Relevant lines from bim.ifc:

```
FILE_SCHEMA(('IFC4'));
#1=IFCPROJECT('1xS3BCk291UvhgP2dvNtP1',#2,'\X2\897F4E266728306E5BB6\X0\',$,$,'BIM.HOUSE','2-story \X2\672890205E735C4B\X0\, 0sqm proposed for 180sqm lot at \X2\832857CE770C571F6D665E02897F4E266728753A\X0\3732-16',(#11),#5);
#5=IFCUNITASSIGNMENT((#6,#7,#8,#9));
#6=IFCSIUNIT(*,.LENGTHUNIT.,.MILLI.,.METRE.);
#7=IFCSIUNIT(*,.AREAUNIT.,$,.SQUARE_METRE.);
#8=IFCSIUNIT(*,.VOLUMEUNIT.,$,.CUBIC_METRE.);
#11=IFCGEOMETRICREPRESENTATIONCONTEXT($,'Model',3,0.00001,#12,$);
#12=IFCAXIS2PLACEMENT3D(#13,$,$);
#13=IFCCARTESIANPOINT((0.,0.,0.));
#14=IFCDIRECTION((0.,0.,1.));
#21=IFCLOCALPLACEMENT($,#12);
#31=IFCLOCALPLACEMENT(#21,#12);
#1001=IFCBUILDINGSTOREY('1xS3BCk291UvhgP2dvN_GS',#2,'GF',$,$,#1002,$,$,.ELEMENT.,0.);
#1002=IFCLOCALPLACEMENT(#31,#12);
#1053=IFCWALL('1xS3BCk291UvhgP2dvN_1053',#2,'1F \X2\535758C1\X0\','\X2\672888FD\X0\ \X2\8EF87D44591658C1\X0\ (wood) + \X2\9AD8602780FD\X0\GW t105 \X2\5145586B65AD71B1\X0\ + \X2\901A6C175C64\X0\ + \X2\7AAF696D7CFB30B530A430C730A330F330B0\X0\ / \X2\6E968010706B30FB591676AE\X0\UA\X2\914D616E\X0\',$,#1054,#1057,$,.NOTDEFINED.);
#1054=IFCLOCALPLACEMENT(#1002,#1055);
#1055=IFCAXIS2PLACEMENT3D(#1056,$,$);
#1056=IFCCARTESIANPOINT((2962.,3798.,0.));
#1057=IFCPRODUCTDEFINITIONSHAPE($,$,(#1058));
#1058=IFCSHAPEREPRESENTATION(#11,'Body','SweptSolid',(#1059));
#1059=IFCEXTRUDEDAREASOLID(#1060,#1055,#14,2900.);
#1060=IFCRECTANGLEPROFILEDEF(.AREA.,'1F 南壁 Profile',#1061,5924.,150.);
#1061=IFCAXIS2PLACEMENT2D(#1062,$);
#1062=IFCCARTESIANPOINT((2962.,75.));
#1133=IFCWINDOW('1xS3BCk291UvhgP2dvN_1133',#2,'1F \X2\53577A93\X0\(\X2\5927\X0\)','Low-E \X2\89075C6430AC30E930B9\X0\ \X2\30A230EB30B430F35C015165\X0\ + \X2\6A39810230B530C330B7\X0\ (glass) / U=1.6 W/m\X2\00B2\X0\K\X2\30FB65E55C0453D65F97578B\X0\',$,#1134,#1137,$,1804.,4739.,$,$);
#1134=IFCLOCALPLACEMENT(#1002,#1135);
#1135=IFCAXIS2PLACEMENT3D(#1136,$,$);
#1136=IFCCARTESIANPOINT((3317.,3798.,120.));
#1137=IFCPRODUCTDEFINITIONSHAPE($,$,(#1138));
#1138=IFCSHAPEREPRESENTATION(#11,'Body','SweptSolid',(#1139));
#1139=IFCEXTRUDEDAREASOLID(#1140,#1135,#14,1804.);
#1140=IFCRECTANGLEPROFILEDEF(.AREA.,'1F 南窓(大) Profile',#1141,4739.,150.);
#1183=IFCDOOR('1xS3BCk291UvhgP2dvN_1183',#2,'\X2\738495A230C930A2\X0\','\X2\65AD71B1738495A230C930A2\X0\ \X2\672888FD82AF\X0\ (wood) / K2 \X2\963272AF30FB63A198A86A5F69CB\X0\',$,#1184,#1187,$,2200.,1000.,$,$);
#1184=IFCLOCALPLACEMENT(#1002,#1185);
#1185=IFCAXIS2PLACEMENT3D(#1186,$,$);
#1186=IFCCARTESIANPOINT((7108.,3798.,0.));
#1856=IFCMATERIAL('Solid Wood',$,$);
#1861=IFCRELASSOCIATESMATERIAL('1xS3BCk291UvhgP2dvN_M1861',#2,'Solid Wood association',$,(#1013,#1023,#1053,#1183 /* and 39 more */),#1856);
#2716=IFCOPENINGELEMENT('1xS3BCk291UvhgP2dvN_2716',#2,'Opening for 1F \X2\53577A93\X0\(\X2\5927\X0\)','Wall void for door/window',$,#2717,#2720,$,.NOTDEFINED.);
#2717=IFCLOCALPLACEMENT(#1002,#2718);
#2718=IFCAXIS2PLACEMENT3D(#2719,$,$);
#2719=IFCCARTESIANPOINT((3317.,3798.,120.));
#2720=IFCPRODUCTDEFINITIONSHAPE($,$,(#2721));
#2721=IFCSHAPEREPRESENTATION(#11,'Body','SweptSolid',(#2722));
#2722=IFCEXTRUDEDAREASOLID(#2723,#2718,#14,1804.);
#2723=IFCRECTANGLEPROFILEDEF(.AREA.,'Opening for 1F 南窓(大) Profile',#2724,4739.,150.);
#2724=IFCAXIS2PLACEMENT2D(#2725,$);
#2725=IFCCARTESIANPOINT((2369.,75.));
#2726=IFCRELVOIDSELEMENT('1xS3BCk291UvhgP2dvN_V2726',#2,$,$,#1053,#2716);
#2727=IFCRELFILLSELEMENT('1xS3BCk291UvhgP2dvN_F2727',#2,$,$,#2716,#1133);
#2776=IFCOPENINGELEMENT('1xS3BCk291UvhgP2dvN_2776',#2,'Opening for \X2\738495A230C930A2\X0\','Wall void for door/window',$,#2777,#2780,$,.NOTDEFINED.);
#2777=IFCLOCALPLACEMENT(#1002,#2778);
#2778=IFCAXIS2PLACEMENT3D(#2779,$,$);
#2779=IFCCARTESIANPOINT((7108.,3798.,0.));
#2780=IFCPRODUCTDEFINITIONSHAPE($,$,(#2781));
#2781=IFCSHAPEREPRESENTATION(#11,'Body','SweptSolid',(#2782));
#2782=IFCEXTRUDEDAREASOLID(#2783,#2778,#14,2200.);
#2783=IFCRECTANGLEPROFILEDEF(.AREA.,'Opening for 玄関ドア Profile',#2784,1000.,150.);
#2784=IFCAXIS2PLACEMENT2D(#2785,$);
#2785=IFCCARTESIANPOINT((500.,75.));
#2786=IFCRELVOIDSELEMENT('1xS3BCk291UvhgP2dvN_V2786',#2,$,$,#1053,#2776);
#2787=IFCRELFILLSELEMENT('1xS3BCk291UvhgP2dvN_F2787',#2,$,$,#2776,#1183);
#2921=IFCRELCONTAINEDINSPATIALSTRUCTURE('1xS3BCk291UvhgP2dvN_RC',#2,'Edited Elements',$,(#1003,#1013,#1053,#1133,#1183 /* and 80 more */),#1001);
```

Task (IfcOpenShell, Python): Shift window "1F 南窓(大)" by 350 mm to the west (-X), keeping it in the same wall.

```python
import ifcopenshell
import ifcopenshell.api.geometry
import ifcopenshell.util.placement

model = ifcopenshell.open("bim.ifc")

window = model.by_guid("1xS3BCk291UvhgP2dvN_1133")
opening = window.FillsVoids[0].RelatingOpeningElement
wall = opening.VoidsElements[0].RelatingBuildingElement

wall_matrix = ifcopenshell.util.placement.get_local_placement(wall.ObjectPlacement)
shift = wall_matrix[:3, 0] * -350.0
before = ifcopenshell.util.placement.get_local_placement(window.ObjectPlacement)[:3, 3].copy()

# The window is not placed relative to its opening, so move both.
for product in (opening, window):
    matrix = ifcopenshell.util.placement.get_local_placement(product.ObjectPlacement)
    matrix[:3, 3] += shift
    ifcopenshell.api.geometry.edit_object_placement(model, product=product, matrix=matrix, is_si=False)

after = ifcopenshell.util.placement.get_local_placement(window.ObjectPlacement)[:3, 3]
print("window moved by", (after - before).round(3) + 0.0)

model.write("bim_rev.ifc")
```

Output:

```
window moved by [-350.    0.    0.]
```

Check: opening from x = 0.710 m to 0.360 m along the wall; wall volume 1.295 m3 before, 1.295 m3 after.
